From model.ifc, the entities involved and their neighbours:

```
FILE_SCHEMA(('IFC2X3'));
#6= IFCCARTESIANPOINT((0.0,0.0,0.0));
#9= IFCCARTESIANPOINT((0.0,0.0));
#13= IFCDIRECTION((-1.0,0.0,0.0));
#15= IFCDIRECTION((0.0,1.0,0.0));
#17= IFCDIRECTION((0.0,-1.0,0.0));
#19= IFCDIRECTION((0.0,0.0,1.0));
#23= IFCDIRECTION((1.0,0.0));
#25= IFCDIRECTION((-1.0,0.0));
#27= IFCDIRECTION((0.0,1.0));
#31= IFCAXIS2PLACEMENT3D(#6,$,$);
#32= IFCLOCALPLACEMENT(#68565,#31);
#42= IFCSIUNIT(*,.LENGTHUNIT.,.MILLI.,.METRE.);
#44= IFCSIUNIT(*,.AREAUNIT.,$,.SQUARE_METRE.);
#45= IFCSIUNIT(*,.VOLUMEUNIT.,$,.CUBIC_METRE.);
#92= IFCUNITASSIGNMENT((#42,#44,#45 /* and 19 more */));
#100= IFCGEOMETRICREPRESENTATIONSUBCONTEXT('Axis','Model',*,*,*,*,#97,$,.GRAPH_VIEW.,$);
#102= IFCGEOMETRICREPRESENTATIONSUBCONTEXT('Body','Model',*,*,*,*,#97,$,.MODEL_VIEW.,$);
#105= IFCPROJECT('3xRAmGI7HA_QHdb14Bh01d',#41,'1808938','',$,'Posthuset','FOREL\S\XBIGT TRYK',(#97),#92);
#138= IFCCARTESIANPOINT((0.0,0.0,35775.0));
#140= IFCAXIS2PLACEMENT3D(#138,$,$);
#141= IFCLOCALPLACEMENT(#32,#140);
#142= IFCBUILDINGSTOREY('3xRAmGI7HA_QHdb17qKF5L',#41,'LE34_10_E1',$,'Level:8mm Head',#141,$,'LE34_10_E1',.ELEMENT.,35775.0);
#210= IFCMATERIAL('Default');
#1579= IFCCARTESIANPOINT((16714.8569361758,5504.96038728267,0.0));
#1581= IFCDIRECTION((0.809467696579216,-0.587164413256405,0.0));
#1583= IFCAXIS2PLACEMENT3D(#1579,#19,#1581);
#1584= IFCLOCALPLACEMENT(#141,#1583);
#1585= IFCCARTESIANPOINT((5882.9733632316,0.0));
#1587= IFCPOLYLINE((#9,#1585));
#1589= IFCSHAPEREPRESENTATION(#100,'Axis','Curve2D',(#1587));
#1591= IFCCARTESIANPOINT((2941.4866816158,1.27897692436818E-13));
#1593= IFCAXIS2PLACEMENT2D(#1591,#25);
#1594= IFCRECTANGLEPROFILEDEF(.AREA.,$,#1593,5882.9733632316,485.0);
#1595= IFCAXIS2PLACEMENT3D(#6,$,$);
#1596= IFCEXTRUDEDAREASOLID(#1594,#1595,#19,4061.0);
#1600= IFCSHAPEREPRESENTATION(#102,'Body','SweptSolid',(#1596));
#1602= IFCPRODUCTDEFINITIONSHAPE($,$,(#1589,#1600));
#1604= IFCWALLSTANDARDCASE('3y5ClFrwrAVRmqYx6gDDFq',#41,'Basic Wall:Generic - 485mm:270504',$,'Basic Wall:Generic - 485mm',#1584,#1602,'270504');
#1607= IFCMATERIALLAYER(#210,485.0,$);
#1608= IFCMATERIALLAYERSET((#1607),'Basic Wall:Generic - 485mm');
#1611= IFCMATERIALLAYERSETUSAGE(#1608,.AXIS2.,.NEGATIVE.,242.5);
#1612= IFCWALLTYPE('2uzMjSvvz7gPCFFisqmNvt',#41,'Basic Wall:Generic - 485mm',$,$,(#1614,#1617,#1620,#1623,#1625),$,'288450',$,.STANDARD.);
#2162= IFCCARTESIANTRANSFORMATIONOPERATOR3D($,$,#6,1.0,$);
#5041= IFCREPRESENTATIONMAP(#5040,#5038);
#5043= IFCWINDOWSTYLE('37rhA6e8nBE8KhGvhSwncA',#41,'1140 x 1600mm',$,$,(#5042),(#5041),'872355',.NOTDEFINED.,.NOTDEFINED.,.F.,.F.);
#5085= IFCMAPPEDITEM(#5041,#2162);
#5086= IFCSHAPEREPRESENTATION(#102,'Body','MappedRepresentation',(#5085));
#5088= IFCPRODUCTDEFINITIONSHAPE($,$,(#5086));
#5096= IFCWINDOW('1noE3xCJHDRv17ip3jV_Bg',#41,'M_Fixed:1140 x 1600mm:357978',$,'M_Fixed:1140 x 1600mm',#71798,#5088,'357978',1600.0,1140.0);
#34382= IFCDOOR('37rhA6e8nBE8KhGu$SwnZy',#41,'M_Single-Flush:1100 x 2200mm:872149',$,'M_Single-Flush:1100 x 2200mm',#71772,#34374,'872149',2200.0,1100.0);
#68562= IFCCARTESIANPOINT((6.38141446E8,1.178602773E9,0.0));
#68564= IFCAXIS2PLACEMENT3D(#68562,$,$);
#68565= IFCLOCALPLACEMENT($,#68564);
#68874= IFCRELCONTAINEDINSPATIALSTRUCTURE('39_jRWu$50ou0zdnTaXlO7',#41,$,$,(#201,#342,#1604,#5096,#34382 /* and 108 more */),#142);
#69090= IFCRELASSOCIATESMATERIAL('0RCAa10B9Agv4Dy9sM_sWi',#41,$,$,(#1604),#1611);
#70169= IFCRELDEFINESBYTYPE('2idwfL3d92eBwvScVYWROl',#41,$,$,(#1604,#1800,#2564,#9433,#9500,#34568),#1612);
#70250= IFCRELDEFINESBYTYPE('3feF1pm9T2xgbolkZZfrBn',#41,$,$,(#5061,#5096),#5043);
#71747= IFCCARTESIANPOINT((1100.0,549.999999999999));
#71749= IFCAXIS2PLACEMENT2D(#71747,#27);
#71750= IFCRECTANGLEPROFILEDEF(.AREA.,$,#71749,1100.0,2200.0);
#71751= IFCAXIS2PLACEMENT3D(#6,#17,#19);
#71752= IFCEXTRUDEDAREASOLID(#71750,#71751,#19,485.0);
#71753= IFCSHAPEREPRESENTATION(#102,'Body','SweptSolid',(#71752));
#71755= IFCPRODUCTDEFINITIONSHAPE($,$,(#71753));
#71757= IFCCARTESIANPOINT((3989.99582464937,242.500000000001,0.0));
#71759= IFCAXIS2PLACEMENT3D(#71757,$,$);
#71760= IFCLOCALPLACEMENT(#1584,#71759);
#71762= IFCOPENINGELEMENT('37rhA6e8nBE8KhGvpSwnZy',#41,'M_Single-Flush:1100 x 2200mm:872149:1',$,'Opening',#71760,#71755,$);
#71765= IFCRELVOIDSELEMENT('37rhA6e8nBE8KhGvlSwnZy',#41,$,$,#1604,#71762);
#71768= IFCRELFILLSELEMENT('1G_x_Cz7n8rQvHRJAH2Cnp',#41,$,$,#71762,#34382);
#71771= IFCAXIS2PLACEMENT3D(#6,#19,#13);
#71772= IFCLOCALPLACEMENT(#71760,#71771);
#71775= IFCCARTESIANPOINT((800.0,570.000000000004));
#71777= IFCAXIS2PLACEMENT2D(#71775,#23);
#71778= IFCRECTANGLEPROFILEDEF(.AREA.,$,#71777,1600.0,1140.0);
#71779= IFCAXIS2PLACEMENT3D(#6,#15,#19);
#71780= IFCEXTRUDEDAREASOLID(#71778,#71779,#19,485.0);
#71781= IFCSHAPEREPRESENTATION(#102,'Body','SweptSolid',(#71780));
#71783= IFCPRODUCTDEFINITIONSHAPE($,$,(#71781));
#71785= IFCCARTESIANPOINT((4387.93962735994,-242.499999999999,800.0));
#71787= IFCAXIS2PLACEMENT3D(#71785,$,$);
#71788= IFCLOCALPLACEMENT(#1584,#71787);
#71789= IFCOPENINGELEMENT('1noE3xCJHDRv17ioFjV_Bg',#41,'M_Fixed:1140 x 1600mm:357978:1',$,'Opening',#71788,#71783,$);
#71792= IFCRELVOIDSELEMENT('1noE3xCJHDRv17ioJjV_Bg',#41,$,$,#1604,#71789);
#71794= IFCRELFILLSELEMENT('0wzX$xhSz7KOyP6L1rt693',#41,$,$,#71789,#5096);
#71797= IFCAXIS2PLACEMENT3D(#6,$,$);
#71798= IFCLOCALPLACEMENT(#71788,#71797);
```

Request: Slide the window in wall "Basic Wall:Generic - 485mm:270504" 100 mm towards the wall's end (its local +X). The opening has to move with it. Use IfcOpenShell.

```python
import ifcopenshell
import ifcopenshell.api.geometry
import ifcopenshell.util.placement
import ifcopenshell.util.unit

model = ifcopenshell.open("model.ifc")
unit_scale = ifcopenshell.util.unit.calculate_unit_scale(model)

window = model.by_guid("1noE3xCJHDRv17ip3jV_Bg")
opening = window.FillsVoids[0].RelatingOpeningElement
wall = opening.VoidsElements[0].RelatingBuildingElement

wall_matrix = ifcopenshell.util.placement.get_local_placement(wall.ObjectPlacement)
shift = wall_matrix[:3, 0] * 0.1 / unit_scale
before = ifcopenshell.util.placement.get_local_placement(window.ObjectPlacement)[:3, 3].copy()

# The window is placed relative to its opening, so it follows when the opening moves.
matrix = ifcopenshell.util.placement.get_local_placement(opening.ObjectPlacement)
matrix[:3, 3] += shift
ifcopenshell.api.geometry.edit_object_placement(
    model, product=opening, matrix=matrix, is_si=False, should_transform_children=True
)

after = ifcopenshell.util.placement.get_local_placement(window.ObjectPlacement)[:3, 3]
print("window moved by", (after - before).round(3) + 0.0)

model.write("model_updated.ifc")
```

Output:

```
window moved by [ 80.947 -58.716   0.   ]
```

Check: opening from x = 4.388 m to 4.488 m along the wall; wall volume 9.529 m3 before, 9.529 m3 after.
